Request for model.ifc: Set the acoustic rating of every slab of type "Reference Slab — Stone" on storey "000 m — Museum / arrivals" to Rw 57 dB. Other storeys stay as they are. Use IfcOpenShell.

First a look at what the model holds.

```python
import ifcopenshell
import ifcopenshell.util.element

model = ifcopenshell.open("model.ifc")
print(model.schema)
storey = next(s for s in model.by_type("IfcBuildingStorey") if s.Name == "000 m — Museum / arrivals")
slabs = [e for e in ifcopenshell.util.element.get_decomposition(storey) if e.is_a("IfcSlab")]
seen = {}
for e in slabs:
    element_type = ifcopenshell.util.element.get_type(e)
    key = (element_type.Name if element_type != e and element_type else None, ifcopenshell.util.element.get_pset(e, "Pset_SlabCommon", "AcousticRating"))
    seen[key] = seen.get(key, 0) + 1
for (name, value), count in sorted(seen.items(), key=str):
    print(count, "x", name, "|", value)
```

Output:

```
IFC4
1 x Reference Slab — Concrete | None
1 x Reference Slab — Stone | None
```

```python
import ifcopenshell
import ifcopenshell.api.pset
import ifcopenshell.util.element

model = ifcopenshell.open("model.ifc")

storey = next(s for s in model.by_type("IfcBuildingStorey") if s.Name == "000 m — Museum / arrivals")
slabs = [e for e in ifcopenshell.util.element.get_decomposition(storey) if e.is_a("IfcSlab")]

count = 0
for e in slabs:
    element_type = ifcopenshell.util.element.get_type(e)
    if element_type in (None, e) or element_type.Name != "Reference Slab — Stone":
        continue
    # add_pset returns the element's existing set when there is one.
    pset = ifcopenshell.api.pset.add_pset(model, product=e, name="Pset_SlabCommon")
    ifcopenshell.api.pset.edit_pset(model, pset=pset, properties={"AcousticRating": "Rw 57 dB"})
    count += 1

print(count, "slabs updated")

model.write("model_updated.ifc")
```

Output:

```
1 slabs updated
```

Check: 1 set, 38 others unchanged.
